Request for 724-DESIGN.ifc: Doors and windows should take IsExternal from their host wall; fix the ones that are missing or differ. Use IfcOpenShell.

First a look at what the model holds.

```python
import ifcopenshell
import ifcopenshell.util.element

model = ifcopenshell.open("724-DESIGN.ifc")
print(model.schema)
seen = {}
for e in model.by_type("IfcDoor") + model.by_type("IfcWindow"):
    if not e.FillsVoids:
        continue
    host = e.FillsVoids[0].RelatingOpeningElement.VoidsElements[0].RelatingBuildingElement
    own = ifcopenshell.util.element.get_pset(e, f"Pset_{e.is_a()[3:].removesuffix('StandardCase')}Common", "IsExternal")
    wall = ifcopenshell.util.element.get_pset(host, "Pset_WallCommon", "IsExternal")
    seen[e.is_a(), own, wall] = seen.get((e.is_a(), own, wall), 0) + 1
for (cls, own, wall), count in sorted(seen.items(), key=str):
    print(count, cls, "IsExternal:", own, "| host wall:", wall)
```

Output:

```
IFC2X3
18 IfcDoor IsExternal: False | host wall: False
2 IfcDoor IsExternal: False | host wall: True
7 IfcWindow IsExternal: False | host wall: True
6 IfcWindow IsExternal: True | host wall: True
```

```python
import ifcopenshell
import ifcopenshell.api.pset
import ifcopenshell.util.element

model = ifcopenshell.open("724-DESIGN.ifc")

count = 0
for ifc_class, pset_name in (("IfcDoor", "Pset_DoorCommon"), ("IfcWindow", "Pset_WindowCommon")):
    for e in model.by_type(ifc_class):
        if not e.FillsVoids:
            continue
        host = e.FillsVoids[0].RelatingOpeningElement.VoidsElements[0].RelatingBuildingElement
        external = ifcopenshell.util.element.get_pset(host, "Pset_WallCommon", "IsExternal")
        if external is None or ifcopenshell.util.element.get_pset(e, pset_name, "IsExternal") == external:
            continue
        pset = ifcopenshell.api.pset.add_pset(model, product=e, name=pset_name)
        ifcopenshell.api.pset.edit_pset(model, pset=pset, properties={"IsExternal": external})
        count += 1

print(count, "updated")

model.write("724-DESIGN-out.ifc")
```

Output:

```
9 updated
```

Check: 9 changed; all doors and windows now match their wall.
